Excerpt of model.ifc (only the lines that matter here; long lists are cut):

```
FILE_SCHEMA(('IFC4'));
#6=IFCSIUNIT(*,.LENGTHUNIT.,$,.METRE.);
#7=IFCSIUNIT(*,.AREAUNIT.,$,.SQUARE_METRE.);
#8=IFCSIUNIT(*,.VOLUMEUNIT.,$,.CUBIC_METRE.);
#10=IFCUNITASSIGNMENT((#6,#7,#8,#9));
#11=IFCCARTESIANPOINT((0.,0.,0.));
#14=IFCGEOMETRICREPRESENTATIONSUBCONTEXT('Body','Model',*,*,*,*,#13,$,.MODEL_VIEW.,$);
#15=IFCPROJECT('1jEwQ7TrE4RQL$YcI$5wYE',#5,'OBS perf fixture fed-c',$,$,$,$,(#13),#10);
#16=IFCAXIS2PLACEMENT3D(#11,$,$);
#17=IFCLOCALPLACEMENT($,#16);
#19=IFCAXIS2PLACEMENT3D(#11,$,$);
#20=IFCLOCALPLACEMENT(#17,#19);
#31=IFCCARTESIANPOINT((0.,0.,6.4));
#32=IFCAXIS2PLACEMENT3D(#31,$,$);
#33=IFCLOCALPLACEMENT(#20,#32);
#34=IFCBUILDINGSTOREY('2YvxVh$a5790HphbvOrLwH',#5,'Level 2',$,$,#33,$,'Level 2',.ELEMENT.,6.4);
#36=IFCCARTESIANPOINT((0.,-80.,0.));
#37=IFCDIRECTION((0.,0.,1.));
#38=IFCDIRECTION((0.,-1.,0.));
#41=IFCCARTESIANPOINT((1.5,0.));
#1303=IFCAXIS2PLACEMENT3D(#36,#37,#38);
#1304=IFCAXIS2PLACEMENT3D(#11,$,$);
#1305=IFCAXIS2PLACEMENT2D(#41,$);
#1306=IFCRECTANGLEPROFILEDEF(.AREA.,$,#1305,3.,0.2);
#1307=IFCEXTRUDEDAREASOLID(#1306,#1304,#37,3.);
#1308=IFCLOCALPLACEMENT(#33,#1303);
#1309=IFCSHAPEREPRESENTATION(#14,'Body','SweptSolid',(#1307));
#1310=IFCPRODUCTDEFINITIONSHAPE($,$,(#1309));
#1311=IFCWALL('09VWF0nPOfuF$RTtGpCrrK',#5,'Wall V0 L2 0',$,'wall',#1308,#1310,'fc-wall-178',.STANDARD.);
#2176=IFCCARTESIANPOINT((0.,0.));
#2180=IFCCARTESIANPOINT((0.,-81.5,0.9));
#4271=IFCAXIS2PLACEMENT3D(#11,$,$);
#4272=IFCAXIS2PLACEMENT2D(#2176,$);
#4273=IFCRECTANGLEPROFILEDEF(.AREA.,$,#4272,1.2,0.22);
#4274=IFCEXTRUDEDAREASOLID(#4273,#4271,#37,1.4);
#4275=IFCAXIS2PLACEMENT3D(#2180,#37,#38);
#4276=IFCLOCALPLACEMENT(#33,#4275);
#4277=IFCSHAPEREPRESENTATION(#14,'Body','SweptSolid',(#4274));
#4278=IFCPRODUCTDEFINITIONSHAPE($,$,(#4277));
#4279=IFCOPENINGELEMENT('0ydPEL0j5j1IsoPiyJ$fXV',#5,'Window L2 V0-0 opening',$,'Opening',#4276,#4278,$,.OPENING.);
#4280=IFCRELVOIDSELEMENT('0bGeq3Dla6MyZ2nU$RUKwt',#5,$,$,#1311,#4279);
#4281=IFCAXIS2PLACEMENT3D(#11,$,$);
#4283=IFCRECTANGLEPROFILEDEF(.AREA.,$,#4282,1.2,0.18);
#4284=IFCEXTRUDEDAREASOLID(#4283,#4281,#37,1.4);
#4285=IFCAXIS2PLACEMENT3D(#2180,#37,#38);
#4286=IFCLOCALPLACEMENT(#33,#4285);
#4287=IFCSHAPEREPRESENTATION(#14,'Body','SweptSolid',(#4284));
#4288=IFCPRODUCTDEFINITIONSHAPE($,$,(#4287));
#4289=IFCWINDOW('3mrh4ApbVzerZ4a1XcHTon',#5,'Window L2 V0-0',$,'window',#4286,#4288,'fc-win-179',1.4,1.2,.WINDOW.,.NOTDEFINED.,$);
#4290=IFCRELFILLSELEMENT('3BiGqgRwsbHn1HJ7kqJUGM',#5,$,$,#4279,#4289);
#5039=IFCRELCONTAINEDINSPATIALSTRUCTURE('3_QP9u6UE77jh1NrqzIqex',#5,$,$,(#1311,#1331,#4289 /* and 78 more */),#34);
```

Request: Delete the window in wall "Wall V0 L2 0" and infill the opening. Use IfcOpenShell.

```python
import ifcopenshell
import ifcopenshell.api.feature
import ifcopenshell.api.root
import ifcopenshell.geom
import ifcopenshell.util.shape

model = ifcopenshell.open("model.ifc")
settings = ifcopenshell.geom.settings()


def volume(element):
    """Net volume in cubic metres, openings subtracted."""
    shape = ifcopenshell.geom.create_shape(settings, element)
    return ifcopenshell.util.shape.get_volume(shape.geometry)


window = model.by_id(4289)
opening = window.FillsVoids[0].RelatingOpeningElement
wall = opening.VoidsElements[0].RelatingBuildingElement
before = volume(wall)

ifcopenshell.api.root.remove_product(model, product=window)
ifcopenshell.api.feature.remove_feature(model, feature=opening)

after = volume(wall)

print(f"wall volume {before:.3f} -> {after:.3f} m3")

model.write("model_updated.ifc")
```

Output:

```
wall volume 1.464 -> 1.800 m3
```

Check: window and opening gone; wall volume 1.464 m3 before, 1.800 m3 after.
